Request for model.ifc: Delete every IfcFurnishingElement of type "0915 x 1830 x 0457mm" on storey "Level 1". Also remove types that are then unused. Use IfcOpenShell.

First a look at what the model holds.

```python
import ifcopenshell
import ifcopenshell.util.element

model = ifcopenshell.open("model.ifc")
print(model.schema)
storey = next(s for s in model.by_type("IfcBuildingStorey") if s.Name == "Level 1")
furniture = [e for e in ifcopenshell.util.element.get_decomposition(storey) if e.is_a("IfcFurnishingElement")]
seen = {}
for e in furniture:
    element_type = ifcopenshell.util.element.get_type(e)
    name = element_type.Name if element_type not in (None, e) else None
    seen[name] = seen.get(name, 0) + 1
for name, count in sorted(seen.items(), key=str):
    print(count, "x", name)
```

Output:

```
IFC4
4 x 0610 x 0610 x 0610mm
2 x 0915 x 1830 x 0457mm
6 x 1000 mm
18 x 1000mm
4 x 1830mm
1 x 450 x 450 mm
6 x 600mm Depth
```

```python
import ifcopenshell
import ifcopenshell.api.root
import ifcopenshell.util.element

model = ifcopenshell.open("model.ifc")

storey = next(s for s in model.by_type("IfcBuildingStorey") if s.Name == "Level 1")
furniture = [e for e in ifcopenshell.util.element.get_decomposition(storey) if e.is_a("IfcFurnishingElement")]
targets = [e for e in furniture if (t := ifcopenshell.util.element.get_type(e)) not in (None, e) and t.Name == "0915 x 1830 x 0457mm"]
types = {ifcopenshell.util.element.get_type(e) for e in targets} - {None, *targets}

for e in targets:
    ifcopenshell.api.root.remove_product(model, product=e)
print(len(targets), "removed")

unused = [t for t in types if not ifcopenshell.util.element.get_types(t)]
for t in unused:
    ifcopenshell.api.root.remove_product(model, product=t)
print(len(unused), "unused types removed")

model.write("model_updated.ifc")
```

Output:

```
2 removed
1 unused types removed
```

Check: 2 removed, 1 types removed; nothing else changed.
